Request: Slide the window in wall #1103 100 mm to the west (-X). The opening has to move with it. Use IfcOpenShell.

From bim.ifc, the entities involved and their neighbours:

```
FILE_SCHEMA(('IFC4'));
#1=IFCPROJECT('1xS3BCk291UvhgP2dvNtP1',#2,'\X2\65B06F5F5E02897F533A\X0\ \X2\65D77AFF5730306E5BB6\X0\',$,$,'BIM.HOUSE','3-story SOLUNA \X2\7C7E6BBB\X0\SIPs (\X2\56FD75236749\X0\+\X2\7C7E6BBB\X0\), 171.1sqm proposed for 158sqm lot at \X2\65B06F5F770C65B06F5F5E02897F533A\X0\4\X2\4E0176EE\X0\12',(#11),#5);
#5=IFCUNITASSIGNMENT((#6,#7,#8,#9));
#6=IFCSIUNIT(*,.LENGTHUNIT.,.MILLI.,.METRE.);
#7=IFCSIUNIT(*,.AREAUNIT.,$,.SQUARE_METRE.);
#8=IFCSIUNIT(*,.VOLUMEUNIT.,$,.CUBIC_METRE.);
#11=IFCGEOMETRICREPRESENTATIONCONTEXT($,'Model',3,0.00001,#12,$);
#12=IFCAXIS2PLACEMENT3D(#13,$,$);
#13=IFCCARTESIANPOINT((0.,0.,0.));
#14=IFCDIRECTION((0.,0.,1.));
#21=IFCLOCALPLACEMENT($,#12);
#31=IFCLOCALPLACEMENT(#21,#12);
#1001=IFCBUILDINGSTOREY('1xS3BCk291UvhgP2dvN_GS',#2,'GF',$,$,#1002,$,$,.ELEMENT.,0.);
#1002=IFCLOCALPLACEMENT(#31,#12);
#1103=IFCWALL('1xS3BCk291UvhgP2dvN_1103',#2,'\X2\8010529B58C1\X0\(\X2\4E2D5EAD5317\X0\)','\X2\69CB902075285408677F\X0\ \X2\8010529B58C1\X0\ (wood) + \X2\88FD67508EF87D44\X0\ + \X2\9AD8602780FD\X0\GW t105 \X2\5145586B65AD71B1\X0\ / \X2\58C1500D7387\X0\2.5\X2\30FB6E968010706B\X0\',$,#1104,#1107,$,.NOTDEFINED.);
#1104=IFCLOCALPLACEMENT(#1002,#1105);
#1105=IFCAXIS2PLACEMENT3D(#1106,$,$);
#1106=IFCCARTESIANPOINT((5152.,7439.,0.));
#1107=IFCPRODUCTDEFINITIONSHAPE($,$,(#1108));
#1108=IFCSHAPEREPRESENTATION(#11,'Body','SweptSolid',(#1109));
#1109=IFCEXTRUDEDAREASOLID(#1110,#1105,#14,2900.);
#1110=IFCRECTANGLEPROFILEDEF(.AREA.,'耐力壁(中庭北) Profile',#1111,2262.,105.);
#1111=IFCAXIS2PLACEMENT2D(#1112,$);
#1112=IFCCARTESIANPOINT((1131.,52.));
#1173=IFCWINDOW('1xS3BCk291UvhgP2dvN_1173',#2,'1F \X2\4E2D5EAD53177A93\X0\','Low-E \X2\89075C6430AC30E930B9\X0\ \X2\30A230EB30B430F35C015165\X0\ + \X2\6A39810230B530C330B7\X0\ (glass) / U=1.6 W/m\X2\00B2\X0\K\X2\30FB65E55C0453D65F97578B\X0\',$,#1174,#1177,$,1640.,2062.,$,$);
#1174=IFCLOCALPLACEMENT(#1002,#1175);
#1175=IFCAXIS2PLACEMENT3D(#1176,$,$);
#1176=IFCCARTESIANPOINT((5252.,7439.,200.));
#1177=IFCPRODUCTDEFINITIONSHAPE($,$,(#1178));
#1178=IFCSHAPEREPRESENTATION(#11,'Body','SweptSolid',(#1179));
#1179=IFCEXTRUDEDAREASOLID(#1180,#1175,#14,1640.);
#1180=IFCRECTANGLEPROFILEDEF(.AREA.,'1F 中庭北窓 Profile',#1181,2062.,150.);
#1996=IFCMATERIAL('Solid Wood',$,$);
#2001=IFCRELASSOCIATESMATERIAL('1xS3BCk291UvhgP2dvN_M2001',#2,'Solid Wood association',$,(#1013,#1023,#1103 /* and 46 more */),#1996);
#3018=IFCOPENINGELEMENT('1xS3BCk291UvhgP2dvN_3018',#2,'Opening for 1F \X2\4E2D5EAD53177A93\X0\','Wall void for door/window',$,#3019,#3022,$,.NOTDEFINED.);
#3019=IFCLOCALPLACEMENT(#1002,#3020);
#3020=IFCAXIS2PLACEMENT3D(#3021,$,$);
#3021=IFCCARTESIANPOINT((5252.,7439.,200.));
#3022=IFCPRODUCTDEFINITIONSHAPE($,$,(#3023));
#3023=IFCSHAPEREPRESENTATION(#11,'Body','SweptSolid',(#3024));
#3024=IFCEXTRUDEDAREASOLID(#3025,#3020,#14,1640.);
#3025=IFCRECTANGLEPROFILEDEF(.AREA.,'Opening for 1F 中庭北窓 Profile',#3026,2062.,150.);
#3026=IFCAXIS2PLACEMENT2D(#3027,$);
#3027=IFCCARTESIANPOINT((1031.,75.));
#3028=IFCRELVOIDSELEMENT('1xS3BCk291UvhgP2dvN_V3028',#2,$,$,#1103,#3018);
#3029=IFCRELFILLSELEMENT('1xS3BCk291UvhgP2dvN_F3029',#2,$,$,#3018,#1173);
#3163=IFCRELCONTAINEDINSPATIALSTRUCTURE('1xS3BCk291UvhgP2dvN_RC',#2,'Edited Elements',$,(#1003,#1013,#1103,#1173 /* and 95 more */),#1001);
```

```python
import ifcopenshell
import ifcopenshell.api.geometry
import ifcopenshell.util.placement
import ifcopenshell.util.unit

model = ifcopenshell.open("bim.ifc")
unit_scale = ifcopenshell.util.unit.calculate_unit_scale(model)

window = model.by_guid("1xS3BCk291UvhgP2dvN_1173")
opening = window.FillsVoids[0].RelatingOpeningElement
wall = opening.VoidsElements[0].RelatingBuildingElement

wall_matrix = ifcopenshell.util.placement.get_local_placement(wall.ObjectPlacement)
shift = wall_matrix[:3, 0] * -0.1 / unit_scale
before = ifcopenshell.util.placement.get_local_placement(window.ObjectPlacement)[:3, 3].copy()

# The window is not placed relative to its opening, so move both.
for product in (opening, window):
    matrix = ifcopenshell.util.placement.get_local_placement(product.ObjectPlacement)
    matrix[:3, 3] += shift
    ifcopenshell.api.geometry.edit_object_placement(model, product=product, matrix=matrix, is_si=False)

after = ifcopenshell.util.placement.get_local_placement(window.ObjectPlacement)[:3, 3]
print("window moved by", (after - before).round(3) + 0.0)

model.write("bim_updated.ifc")
```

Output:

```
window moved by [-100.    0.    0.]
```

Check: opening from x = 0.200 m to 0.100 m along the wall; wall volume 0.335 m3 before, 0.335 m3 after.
